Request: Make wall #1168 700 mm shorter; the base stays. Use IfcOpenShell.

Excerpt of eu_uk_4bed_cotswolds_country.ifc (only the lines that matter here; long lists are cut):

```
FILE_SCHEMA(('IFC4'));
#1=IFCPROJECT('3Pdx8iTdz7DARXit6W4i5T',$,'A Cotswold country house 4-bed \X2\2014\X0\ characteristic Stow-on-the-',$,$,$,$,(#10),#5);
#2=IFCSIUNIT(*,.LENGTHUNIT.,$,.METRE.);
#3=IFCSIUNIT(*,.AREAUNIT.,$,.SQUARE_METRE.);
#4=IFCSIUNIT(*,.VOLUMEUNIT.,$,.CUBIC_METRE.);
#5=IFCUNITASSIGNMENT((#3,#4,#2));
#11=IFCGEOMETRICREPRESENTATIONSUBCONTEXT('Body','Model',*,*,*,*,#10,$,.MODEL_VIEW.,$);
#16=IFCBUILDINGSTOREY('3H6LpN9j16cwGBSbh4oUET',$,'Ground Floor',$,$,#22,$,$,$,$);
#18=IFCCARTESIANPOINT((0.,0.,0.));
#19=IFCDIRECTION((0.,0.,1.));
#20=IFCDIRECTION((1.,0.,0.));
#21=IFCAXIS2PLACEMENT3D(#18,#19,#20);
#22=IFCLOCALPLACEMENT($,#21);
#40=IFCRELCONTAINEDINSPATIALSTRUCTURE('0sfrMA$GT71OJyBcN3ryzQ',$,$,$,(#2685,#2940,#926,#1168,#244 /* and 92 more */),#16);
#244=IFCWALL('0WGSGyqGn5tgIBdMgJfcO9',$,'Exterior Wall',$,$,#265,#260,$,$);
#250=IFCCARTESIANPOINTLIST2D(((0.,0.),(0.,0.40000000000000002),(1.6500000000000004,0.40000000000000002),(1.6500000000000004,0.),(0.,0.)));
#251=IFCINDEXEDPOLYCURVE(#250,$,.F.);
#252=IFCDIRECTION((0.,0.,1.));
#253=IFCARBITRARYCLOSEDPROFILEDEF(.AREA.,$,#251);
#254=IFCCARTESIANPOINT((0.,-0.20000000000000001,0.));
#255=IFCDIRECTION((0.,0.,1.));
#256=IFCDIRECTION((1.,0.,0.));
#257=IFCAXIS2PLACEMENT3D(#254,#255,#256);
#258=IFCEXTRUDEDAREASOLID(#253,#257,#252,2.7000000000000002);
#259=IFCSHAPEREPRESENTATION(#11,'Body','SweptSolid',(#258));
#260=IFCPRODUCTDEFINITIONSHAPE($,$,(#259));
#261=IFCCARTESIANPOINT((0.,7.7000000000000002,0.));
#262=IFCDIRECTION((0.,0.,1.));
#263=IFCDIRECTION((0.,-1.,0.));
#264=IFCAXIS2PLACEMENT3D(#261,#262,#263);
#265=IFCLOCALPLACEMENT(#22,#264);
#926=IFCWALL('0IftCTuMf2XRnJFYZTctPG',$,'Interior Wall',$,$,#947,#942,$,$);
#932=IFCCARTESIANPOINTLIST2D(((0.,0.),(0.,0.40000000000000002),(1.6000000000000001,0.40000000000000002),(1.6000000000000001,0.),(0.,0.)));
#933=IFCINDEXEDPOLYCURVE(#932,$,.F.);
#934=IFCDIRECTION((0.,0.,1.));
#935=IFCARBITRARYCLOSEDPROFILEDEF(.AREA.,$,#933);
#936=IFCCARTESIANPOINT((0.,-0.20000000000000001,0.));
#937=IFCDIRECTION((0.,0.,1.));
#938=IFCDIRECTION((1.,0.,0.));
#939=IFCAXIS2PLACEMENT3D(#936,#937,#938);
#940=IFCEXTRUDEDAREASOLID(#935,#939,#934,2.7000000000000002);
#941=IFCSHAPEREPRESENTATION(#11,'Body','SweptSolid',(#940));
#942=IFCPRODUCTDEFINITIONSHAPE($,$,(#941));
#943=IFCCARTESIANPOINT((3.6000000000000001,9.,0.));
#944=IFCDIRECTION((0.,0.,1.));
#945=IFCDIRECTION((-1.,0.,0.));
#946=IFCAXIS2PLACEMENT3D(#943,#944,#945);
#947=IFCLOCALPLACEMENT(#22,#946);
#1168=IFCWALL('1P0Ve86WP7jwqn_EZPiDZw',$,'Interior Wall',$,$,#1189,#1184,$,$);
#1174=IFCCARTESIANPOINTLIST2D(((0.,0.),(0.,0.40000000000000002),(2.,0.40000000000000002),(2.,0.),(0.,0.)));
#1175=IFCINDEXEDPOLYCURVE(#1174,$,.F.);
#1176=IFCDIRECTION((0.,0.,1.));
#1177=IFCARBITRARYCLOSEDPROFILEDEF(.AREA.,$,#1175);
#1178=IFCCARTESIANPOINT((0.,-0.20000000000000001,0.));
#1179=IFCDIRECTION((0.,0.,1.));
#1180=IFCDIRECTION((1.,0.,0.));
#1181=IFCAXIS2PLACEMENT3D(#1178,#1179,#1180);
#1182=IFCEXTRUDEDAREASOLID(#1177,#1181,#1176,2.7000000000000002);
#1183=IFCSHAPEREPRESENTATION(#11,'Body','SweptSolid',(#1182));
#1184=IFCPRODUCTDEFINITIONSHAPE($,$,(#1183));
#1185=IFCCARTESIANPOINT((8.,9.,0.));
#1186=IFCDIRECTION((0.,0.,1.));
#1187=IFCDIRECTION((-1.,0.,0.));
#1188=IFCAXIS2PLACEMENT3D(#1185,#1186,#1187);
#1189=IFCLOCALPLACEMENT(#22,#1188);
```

```python
import ifcopenshell
import ifcopenshell.geom
import ifcopenshell.util.representation
import ifcopenshell.util.shape
import ifcopenshell.util.unit

model = ifcopenshell.open("eu_uk_4bed_cotswolds_country.ifc")
unit_scale = ifcopenshell.util.unit.calculate_unit_scale(model)
settings = ifcopenshell.geom.settings()


def volume(element):
    """Net volume in cubic metres, openings subtracted."""
    shape = ifcopenshell.geom.create_shape(settings, element)
    return ifcopenshell.util.shape.get_volume(shape.geometry)


wall = model.by_guid("1P0Ve86WP7jwqn_EZPiDZw")
before = volume(wall)

body = ifcopenshell.util.representation.get_representation(wall, "Model", "Body")
solid = body.Items[0]
old_height = solid.Depth
solid.Depth -= 0.7 / unit_scale
after = volume(wall)

print(f"height {old_height:g} -> {solid.Depth:g}, volume {before:.3f} -> {after:.3f} m3")

model.write("eu_uk_4bed_cotswolds_country_edited.ifc")
```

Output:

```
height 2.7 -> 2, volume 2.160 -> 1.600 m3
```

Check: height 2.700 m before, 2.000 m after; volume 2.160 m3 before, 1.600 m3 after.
